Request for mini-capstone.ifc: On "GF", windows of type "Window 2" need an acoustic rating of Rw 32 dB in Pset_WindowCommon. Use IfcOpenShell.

First a look at what the model holds.

```python
import ifcopenshell
import ifcopenshell.util.element

model = ifcopenshell.open("mini-capstone.ifc")
print(model.schema)
storey = next(s for s in model.by_type("IfcBuildingStorey") if s.Name == "GF")
windows = [e for e in ifcopenshell.util.element.get_decomposition(storey) if e.is_a("IfcWindow")]
seen = {}
for e in windows:
    element_type = ifcopenshell.util.element.get_type(e)
    key = (element_type.Name if element_type != e and element_type else None, ifcopenshell.util.element.get_pset(e, "Pset_WindowCommon", "AcousticRating"))
    seen[key] = seen.get(key, 0) + 1
for (name, value), count in sorted(seen.items(), key=str):
    print(count, "x", name, "|", value)
```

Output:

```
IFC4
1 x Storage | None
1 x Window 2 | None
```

```python
import ifcopenshell
import ifcopenshell.api.pset
import ifcopenshell.util.element

model = ifcopenshell.open("mini-capstone.ifc")

storey = next(s for s in model.by_type("IfcBuildingStorey") if s.Name == "GF")
windows = [e for e in ifcopenshell.util.element.get_decomposition(storey) if e.is_a("IfcWindow")]

count = 0
for e in windows:
    element_type = ifcopenshell.util.element.get_type(e)
    if element_type in (None, e) or element_type.Name != "Window 2":
        continue
    # add_pset returns the element's existing set when there is one.
    pset = ifcopenshell.api.pset.add_pset(model, product=e, name="Pset_WindowCommon")
    ifcopenshell.api.pset.edit_pset(model, pset=pset, properties={"AcousticRating": "Rw 32 dB"})
    count += 1

print(count, "windows updated")

model.write("mini-capstone_rev.ifc")
```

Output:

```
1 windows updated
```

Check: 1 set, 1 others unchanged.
